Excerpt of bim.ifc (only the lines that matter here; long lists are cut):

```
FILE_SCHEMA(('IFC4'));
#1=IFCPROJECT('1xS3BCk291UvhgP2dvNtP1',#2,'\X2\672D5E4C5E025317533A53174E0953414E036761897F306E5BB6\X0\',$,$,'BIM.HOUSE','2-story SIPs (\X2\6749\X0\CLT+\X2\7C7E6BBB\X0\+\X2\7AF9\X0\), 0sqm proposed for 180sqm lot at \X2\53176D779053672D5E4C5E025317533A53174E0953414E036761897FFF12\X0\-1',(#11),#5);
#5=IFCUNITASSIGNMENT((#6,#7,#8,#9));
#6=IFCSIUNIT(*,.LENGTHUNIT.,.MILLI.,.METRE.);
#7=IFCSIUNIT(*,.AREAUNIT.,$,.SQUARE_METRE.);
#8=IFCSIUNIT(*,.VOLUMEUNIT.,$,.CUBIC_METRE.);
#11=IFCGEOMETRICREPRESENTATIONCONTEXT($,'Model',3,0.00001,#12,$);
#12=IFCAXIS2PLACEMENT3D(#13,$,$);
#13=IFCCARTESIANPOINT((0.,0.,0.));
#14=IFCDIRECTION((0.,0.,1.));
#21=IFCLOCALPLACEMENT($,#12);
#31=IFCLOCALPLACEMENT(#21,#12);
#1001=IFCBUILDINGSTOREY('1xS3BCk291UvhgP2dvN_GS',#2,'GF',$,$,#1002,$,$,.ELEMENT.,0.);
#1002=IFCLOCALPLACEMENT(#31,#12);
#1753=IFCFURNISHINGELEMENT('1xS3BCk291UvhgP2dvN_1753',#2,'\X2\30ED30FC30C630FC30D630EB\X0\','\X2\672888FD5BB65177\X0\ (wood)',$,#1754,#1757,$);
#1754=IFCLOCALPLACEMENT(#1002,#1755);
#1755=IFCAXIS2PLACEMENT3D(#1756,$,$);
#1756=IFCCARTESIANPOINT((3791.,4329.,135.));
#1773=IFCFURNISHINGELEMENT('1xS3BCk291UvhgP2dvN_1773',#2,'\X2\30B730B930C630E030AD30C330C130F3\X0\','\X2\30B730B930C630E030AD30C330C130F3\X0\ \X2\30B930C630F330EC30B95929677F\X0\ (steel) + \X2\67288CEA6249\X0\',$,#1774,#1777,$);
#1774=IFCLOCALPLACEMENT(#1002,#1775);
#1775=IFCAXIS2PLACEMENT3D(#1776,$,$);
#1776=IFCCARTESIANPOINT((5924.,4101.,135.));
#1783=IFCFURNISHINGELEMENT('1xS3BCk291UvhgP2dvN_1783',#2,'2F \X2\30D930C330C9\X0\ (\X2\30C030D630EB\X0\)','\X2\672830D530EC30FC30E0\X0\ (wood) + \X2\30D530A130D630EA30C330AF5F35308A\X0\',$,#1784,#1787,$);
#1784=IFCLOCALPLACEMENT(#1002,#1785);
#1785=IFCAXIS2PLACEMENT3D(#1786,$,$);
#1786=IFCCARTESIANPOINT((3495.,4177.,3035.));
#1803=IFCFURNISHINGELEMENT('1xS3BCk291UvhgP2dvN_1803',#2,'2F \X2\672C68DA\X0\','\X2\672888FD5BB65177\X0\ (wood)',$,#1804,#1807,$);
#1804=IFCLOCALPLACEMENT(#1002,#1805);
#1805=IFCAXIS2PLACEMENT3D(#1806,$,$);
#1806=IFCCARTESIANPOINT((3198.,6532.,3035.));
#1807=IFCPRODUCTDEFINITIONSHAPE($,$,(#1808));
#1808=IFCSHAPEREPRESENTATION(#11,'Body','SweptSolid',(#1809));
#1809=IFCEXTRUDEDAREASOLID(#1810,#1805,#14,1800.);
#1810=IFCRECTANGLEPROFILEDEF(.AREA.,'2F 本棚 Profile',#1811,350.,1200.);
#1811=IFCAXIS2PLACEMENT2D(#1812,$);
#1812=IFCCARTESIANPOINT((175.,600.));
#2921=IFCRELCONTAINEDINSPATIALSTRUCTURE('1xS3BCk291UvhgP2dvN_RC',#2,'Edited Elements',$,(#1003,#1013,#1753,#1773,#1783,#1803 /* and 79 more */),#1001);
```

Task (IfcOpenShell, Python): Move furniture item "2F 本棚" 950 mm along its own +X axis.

```python
import ifcopenshell
import ifcopenshell.api.geometry
import ifcopenshell.util.placement

model = ifcopenshell.open("bim.ifc")

item = model.by_id(1803)
matrix = ifcopenshell.util.placement.get_local_placement(item.ObjectPlacement)
matrix[:3, 3] += matrix[:3, 0] * 950.0
ifcopenshell.api.geometry.edit_object_placement(model, product=item, matrix=matrix, is_si=False)

print(ifcopenshell.util.placement.get_local_placement(item.ObjectPlacement).round(3) + 0.0)

model.write("bim_v2.ifc")
```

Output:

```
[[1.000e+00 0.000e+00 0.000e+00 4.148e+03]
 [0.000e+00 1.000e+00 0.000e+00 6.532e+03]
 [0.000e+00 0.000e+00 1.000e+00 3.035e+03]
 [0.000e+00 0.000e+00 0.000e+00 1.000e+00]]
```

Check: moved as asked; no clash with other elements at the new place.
